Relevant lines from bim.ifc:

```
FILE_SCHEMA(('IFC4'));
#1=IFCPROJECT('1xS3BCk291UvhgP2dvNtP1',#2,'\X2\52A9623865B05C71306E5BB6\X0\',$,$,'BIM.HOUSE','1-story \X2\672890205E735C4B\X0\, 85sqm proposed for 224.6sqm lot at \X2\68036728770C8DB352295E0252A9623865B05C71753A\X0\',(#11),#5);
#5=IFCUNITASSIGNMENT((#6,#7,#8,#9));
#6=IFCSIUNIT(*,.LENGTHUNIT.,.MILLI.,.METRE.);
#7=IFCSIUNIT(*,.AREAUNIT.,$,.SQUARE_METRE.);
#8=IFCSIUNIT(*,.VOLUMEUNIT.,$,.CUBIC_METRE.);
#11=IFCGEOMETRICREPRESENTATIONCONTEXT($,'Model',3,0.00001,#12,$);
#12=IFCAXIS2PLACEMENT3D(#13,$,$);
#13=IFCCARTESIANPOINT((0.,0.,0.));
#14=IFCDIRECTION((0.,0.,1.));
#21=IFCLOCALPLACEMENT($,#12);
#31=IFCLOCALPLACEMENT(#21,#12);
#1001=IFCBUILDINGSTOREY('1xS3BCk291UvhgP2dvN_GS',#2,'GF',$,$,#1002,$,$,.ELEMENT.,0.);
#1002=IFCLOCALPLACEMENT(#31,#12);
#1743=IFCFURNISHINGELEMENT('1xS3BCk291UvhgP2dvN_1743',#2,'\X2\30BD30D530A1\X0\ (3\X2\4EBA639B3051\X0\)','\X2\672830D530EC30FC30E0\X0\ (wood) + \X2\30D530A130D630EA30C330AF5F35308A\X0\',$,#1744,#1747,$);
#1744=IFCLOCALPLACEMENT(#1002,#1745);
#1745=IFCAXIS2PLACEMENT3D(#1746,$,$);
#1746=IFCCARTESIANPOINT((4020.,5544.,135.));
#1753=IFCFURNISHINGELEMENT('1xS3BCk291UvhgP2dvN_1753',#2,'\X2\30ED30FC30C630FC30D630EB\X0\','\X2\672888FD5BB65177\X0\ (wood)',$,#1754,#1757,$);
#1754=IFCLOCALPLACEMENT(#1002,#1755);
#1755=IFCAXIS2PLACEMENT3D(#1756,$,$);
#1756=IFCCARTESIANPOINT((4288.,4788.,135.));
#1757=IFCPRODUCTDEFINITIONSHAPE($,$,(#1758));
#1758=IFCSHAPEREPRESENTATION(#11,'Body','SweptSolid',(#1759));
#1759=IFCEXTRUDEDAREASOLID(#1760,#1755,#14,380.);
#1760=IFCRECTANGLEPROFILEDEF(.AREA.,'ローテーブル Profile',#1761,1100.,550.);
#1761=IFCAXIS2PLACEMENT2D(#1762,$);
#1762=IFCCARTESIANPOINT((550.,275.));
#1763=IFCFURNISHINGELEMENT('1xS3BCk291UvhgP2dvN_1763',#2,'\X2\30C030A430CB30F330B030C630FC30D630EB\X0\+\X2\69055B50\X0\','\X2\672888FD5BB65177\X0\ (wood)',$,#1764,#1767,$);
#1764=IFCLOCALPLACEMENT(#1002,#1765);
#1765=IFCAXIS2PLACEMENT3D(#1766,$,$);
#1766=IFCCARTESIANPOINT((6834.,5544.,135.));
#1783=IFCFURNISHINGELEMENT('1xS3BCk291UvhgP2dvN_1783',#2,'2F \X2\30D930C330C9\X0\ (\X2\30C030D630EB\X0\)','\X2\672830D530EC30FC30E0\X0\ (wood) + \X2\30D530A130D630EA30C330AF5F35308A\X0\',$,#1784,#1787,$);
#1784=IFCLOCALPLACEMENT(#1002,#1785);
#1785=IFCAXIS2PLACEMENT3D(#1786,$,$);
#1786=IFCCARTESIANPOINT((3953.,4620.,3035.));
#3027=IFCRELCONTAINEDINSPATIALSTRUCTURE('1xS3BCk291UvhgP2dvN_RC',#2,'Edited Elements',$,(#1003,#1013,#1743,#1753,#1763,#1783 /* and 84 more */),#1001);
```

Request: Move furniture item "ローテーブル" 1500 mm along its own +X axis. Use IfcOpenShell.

```python
import ifcopenshell
import ifcopenshell.api.geometry
import ifcopenshell.util.placement
import ifcopenshell.util.unit

model = ifcopenshell.open("bim.ifc")
unit_scale = ifcopenshell.util.unit.calculate_unit_scale(model)

item = model.by_id(1753)
matrix = ifcopenshell.util.placement.get_local_placement(item.ObjectPlacement)
matrix[:3, 3] += matrix[:3, 0] * 1.5 / unit_scale
ifcopenshell.api.geometry.edit_object_placement(model, product=item, matrix=matrix, is_si=False)

print(ifcopenshell.util.placement.get_local_placement(item.ObjectPlacement).round(3) + 0.0)

model.write("bim_updated.ifc")
```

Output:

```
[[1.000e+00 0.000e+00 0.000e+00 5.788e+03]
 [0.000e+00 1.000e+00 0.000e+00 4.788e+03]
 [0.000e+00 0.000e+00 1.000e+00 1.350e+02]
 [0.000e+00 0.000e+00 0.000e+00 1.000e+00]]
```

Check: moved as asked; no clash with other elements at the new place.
